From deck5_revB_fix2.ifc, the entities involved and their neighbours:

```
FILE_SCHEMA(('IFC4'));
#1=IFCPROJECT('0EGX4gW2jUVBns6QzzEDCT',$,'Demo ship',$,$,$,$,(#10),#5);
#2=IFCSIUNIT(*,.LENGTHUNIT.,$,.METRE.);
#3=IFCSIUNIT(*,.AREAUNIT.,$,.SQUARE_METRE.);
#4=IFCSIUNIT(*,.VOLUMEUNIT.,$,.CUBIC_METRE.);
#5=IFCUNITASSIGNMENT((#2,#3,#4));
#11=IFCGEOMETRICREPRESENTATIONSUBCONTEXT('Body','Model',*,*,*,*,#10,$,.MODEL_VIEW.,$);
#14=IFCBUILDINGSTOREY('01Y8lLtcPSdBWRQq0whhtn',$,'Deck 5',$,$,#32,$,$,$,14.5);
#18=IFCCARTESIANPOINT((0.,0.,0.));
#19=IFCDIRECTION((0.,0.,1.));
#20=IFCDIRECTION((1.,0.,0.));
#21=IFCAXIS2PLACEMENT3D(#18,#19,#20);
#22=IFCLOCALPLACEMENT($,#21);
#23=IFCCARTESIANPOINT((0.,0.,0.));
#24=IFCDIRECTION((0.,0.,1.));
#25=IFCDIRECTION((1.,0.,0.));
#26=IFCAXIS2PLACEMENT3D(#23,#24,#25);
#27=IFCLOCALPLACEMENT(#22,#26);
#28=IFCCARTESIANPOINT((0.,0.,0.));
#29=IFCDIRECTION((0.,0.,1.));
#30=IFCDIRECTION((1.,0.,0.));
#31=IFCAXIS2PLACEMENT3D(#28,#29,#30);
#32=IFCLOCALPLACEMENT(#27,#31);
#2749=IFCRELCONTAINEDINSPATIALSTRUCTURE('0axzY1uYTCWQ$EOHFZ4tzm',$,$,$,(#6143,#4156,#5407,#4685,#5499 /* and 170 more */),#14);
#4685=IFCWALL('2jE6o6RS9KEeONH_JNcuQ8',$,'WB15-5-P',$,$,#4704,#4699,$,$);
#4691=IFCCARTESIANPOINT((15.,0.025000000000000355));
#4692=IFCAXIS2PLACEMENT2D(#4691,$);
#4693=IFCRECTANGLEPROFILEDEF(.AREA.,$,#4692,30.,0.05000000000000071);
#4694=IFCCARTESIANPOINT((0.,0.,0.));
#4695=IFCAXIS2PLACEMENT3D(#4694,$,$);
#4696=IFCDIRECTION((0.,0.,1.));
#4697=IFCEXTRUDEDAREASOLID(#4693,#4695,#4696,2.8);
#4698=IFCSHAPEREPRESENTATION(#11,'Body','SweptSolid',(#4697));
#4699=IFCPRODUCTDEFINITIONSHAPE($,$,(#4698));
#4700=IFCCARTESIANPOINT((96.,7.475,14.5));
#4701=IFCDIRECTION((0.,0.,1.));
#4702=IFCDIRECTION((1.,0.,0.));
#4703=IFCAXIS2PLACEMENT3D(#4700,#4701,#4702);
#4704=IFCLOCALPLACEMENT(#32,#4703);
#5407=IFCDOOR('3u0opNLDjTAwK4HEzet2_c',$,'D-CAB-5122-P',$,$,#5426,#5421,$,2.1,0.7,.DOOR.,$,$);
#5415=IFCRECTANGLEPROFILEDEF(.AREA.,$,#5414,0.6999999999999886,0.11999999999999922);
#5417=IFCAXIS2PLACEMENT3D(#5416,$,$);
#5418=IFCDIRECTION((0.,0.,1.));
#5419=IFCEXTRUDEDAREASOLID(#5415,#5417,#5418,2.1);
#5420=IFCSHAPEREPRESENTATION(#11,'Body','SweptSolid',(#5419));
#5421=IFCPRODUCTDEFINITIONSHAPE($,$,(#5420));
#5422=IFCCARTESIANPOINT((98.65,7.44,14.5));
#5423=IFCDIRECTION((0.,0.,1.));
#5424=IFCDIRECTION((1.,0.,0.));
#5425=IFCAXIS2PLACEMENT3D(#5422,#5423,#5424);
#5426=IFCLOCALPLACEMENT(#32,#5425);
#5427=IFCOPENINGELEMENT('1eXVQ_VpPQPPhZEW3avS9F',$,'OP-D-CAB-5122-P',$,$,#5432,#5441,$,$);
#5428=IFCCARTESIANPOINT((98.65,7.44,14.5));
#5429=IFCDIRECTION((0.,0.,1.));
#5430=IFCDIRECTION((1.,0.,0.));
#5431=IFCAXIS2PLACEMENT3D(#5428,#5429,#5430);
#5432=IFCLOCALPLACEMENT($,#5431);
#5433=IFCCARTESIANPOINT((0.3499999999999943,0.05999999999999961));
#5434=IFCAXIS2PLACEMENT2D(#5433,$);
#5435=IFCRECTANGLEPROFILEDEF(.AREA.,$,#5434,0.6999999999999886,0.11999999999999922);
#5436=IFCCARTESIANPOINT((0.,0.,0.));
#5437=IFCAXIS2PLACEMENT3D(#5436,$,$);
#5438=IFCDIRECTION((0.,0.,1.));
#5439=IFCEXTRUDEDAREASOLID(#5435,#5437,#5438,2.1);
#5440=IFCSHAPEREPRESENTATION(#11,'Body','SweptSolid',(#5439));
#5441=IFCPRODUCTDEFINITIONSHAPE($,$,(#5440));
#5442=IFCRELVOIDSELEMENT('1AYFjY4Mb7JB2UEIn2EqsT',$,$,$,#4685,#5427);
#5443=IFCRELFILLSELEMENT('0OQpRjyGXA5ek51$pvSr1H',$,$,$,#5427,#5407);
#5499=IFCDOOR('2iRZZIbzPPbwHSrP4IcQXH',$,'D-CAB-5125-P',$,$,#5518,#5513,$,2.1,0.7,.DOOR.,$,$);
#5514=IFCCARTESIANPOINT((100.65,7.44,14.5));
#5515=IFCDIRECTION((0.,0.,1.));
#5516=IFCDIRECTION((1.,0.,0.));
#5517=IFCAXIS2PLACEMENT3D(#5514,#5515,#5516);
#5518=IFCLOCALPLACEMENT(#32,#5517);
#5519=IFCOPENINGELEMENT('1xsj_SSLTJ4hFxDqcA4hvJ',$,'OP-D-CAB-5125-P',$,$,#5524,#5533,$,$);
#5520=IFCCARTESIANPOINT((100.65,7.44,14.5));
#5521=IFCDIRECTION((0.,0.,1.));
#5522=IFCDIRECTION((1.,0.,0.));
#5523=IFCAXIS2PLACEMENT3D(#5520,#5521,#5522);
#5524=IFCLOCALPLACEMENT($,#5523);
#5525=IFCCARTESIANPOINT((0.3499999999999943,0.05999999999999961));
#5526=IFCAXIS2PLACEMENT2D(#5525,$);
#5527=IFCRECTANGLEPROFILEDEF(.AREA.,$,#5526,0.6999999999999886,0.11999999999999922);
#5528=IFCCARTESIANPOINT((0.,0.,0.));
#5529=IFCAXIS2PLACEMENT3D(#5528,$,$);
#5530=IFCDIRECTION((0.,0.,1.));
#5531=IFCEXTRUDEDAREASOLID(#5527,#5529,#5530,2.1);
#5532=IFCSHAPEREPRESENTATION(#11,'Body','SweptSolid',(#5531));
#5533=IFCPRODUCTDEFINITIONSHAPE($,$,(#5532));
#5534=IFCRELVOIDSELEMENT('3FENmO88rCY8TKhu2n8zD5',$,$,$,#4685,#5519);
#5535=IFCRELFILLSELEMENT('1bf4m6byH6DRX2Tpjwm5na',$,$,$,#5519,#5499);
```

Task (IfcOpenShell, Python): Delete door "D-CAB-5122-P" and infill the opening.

```python
import ifcopenshell
import ifcopenshell.api.feature
import ifcopenshell.api.root
import ifcopenshell.geom
import ifcopenshell.util.shape

model = ifcopenshell.open("deck5_revB_fix2.ifc")
settings = ifcopenshell.geom.settings()


def volume(element):
    """Net volume in cubic metres, openings subtracted."""
    shape = ifcopenshell.geom.create_shape(settings, element)
    return ifcopenshell.util.shape.get_volume(shape.geometry)


door = model.by_guid("3u0opNLDjTAwK4HEzet2_c")
opening = door.FillsVoids[0].RelatingOpeningElement
wall = opening.VoidsElements[0].RelatingBuildingElement
before = volume(wall)

ifcopenshell.api.root.remove_product(model, product=door)
ifcopenshell.api.feature.remove_feature(model, feature=opening)

after = volume(wall)

print(f"wall volume {before:.3f} -> {after:.3f} m3")

model.write("deck5_revB_fix2_v2.ifc")
```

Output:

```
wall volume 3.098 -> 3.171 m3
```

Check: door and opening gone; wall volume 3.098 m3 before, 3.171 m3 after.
